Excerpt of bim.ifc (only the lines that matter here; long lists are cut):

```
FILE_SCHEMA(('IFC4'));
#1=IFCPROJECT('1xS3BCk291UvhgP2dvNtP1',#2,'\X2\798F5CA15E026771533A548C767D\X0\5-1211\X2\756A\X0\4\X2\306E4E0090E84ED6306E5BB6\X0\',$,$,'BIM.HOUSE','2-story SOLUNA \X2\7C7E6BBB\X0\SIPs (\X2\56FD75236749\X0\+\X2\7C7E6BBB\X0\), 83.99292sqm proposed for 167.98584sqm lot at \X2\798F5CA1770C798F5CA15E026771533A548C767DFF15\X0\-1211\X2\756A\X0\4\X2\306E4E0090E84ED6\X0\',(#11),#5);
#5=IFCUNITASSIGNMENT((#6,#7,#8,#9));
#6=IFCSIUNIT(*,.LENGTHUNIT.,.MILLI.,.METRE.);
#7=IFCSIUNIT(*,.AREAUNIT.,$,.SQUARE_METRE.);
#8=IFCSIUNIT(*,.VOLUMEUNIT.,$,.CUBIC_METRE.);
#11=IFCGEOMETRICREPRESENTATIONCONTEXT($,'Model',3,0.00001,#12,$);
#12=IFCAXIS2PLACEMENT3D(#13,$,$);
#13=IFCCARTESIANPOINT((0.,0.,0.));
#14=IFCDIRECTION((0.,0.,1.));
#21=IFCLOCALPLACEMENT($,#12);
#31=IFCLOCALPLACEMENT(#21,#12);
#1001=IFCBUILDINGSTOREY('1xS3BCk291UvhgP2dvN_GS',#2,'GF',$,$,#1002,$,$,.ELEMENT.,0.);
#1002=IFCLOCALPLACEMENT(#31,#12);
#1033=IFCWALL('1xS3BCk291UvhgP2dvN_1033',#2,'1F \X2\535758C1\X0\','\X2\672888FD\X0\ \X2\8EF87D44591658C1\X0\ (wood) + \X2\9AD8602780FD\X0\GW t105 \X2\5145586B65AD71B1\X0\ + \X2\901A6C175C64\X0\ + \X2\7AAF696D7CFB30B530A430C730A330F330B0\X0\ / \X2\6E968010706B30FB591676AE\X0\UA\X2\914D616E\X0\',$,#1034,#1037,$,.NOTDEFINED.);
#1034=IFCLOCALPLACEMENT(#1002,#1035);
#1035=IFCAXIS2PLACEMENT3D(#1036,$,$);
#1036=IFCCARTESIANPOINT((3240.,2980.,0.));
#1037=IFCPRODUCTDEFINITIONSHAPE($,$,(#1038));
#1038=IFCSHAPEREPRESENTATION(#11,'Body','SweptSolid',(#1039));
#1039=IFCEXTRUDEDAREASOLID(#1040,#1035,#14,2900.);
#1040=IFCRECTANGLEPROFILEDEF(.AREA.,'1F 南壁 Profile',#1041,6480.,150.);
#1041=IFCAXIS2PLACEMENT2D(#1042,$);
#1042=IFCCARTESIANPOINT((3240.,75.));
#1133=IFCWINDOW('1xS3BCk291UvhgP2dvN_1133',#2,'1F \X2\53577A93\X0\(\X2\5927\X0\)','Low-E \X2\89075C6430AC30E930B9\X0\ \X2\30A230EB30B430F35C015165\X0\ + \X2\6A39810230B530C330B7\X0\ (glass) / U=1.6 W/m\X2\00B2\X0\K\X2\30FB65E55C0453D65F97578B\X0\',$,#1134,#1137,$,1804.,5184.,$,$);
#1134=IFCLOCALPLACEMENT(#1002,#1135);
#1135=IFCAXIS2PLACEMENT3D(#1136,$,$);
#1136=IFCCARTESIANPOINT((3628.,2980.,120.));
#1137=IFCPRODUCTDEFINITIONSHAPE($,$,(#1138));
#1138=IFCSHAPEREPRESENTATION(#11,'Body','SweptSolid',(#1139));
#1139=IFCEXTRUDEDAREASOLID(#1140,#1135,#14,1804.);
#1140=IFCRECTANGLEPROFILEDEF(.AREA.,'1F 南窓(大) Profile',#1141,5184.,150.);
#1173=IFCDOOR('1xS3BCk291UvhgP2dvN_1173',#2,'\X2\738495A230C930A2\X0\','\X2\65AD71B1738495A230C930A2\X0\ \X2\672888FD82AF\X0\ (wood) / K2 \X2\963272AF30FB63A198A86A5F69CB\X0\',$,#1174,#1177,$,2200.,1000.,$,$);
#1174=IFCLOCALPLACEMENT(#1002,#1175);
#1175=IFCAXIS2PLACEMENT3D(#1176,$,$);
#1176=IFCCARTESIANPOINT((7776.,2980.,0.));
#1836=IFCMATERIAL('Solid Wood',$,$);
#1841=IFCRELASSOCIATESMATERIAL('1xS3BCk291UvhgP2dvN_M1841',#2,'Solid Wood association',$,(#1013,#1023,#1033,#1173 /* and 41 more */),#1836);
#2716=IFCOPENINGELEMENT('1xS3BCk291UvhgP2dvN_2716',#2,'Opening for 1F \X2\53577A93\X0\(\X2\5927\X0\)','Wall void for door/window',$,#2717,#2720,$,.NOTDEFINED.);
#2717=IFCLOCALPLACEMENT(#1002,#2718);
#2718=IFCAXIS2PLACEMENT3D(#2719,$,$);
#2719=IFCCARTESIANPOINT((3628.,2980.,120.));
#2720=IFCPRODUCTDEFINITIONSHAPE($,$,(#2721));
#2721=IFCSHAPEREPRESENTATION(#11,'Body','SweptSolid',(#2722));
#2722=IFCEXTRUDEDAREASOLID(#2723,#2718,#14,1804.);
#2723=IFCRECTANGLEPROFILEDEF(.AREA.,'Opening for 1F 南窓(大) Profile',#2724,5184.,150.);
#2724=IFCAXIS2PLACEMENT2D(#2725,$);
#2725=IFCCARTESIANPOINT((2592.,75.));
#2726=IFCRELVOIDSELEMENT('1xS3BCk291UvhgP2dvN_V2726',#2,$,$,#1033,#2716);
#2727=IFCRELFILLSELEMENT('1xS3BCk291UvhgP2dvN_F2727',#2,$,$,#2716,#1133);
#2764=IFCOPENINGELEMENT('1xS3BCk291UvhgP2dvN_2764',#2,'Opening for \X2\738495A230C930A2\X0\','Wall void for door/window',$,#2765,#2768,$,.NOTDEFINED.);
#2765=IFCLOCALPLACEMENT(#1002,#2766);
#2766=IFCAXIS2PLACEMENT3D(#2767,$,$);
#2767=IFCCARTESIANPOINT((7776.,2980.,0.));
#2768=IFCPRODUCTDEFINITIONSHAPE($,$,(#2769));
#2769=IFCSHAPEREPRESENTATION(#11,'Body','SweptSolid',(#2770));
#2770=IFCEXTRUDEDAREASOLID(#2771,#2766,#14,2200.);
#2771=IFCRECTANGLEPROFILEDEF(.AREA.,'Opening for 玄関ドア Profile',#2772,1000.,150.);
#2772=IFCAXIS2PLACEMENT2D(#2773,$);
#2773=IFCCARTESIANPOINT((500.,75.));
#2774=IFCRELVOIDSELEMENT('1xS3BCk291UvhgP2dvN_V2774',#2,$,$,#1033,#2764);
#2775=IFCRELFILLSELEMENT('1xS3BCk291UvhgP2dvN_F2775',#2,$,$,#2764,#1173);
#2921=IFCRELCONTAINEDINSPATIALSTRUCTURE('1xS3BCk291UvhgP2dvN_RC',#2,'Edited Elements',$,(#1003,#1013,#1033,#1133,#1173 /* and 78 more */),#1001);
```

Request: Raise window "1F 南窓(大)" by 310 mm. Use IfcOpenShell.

```python
import numpy as np
import ifcopenshell
import ifcopenshell.api.geometry
import ifcopenshell.util.placement
import ifcopenshell.util.unit

model = ifcopenshell.open("bim.ifc")
unit_scale = ifcopenshell.util.unit.calculate_unit_scale(model)

window = model.by_id(1133)
opening = window.FillsVoids[0].RelatingOpeningElement
dz = 0.31 / unit_scale

shift = np.array([0.0, 0.0, dz])
# The window is not placed relative to its opening, so move both.
for product in (opening, window):
    matrix = ifcopenshell.util.placement.get_local_placement(product.ObjectPlacement)
    matrix[:3, 3] += shift
    ifcopenshell.api.geometry.edit_object_placement(model, product=product, matrix=matrix, is_si=False)

print(f"moved by {dz * unit_scale:+.3f} m")

model.write("bim_edited.ifc")
```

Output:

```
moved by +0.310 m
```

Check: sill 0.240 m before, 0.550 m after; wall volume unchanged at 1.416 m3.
